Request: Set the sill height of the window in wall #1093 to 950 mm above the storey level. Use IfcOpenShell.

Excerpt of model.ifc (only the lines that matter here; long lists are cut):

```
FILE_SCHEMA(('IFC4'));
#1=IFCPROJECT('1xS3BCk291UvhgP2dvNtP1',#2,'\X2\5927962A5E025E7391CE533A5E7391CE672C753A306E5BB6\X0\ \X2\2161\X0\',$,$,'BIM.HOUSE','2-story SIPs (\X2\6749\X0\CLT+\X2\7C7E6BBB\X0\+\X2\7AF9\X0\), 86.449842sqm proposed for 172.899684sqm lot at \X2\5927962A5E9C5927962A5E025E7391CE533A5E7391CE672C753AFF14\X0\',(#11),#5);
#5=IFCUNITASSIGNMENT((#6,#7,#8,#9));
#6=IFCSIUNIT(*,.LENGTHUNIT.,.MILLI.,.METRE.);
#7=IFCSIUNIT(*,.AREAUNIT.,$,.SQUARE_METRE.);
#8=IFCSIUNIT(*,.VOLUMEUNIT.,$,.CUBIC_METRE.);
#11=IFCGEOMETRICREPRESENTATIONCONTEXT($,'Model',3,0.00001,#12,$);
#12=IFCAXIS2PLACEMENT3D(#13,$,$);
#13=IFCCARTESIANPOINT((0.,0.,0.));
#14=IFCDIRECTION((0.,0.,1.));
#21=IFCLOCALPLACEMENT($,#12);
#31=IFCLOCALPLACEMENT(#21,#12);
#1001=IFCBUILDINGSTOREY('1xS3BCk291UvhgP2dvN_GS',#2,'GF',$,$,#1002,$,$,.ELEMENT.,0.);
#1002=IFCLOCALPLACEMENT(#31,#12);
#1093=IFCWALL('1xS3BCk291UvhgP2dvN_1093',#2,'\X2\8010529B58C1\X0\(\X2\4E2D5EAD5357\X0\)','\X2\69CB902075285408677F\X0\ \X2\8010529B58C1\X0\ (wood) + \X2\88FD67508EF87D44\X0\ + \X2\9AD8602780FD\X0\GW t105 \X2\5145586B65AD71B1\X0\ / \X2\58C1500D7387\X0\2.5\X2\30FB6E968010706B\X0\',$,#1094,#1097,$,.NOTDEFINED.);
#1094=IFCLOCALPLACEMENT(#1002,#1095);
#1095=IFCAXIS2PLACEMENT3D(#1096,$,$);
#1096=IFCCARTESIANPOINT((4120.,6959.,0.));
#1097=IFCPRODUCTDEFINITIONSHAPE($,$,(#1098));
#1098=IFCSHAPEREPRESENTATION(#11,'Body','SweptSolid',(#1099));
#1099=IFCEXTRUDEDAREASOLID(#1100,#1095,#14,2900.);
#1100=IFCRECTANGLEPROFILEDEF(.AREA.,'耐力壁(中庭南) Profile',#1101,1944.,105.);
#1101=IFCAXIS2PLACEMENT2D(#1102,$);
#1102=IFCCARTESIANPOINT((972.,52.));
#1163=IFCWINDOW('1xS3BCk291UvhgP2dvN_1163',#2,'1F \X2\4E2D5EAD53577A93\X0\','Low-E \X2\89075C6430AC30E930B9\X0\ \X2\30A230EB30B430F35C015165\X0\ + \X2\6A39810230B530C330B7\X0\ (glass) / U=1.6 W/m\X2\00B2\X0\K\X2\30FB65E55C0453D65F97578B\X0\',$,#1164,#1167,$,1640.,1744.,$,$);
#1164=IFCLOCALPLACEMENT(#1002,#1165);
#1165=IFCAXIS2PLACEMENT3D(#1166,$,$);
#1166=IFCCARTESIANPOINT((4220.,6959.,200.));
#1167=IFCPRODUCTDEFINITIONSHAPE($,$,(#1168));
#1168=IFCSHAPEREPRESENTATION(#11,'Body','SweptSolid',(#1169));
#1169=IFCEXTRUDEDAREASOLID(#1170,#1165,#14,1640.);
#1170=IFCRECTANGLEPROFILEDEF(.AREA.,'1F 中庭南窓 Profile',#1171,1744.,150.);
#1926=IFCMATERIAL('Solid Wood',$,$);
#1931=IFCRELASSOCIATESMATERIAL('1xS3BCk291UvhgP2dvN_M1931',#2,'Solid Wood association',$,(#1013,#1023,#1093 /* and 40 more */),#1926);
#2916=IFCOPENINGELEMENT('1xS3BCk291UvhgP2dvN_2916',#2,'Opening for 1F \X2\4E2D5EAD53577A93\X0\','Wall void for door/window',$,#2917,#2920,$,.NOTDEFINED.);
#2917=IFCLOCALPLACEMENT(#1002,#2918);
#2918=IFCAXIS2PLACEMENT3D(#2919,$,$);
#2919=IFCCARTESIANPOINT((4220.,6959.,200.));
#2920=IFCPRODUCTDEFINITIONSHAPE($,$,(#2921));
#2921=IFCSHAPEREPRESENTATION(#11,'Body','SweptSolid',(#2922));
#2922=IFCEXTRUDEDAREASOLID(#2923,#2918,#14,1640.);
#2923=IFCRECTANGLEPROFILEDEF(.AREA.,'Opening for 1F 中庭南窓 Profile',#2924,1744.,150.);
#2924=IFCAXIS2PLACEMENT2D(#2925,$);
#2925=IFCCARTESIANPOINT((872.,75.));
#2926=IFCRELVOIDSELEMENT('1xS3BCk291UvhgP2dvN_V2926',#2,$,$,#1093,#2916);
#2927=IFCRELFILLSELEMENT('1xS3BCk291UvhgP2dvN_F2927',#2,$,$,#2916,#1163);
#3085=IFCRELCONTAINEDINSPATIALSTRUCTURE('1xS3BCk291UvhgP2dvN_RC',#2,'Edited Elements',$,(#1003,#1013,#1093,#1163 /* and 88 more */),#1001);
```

```python
import numpy as np
import ifcopenshell
import ifcopenshell.api.geometry
import ifcopenshell.geom
import ifcopenshell.util.element
import ifcopenshell.util.placement
import ifcopenshell.util.shape
import ifcopenshell.util.unit

model = ifcopenshell.open("model.ifc")
unit_scale = ifcopenshell.util.unit.calculate_unit_scale(model)

window = model.by_guid("1xS3BCk291UvhgP2dvN_1163")
opening = window.FillsVoids[0].RelatingOpeningElement
storey = ifcopenshell.util.element.get_container(window, ifc_class="IfcBuildingStorey")
level = ifcopenshell.util.placement.get_local_placement(storey.ObjectPlacement)[2, 3]

# The opening's origin need not be at the sill, so measure its lowest point.
shape = ifcopenshell.geom.create_shape(ifcopenshell.geom.settings(), opening)
bottom = ifcopenshell.util.shape.get_shape_bottom_elevation(shape, shape.geometry) / unit_scale
dz = level + 0.95 / unit_scale - bottom

shift = np.array([0.0, 0.0, dz])
# The window is not placed relative to its opening, so move both.
for product in (opening, window):
    matrix = ifcopenshell.util.placement.get_local_placement(product.ObjectPlacement)
    matrix[:3, 3] += shift
    ifcopenshell.api.geometry.edit_object_placement(model, product=product, matrix=matrix, is_si=False)

print(f"moved by {dz * unit_scale:+.3f} m")

model.write("model_rev.ifc")
```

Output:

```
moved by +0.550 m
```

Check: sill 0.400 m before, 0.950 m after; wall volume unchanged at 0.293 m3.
